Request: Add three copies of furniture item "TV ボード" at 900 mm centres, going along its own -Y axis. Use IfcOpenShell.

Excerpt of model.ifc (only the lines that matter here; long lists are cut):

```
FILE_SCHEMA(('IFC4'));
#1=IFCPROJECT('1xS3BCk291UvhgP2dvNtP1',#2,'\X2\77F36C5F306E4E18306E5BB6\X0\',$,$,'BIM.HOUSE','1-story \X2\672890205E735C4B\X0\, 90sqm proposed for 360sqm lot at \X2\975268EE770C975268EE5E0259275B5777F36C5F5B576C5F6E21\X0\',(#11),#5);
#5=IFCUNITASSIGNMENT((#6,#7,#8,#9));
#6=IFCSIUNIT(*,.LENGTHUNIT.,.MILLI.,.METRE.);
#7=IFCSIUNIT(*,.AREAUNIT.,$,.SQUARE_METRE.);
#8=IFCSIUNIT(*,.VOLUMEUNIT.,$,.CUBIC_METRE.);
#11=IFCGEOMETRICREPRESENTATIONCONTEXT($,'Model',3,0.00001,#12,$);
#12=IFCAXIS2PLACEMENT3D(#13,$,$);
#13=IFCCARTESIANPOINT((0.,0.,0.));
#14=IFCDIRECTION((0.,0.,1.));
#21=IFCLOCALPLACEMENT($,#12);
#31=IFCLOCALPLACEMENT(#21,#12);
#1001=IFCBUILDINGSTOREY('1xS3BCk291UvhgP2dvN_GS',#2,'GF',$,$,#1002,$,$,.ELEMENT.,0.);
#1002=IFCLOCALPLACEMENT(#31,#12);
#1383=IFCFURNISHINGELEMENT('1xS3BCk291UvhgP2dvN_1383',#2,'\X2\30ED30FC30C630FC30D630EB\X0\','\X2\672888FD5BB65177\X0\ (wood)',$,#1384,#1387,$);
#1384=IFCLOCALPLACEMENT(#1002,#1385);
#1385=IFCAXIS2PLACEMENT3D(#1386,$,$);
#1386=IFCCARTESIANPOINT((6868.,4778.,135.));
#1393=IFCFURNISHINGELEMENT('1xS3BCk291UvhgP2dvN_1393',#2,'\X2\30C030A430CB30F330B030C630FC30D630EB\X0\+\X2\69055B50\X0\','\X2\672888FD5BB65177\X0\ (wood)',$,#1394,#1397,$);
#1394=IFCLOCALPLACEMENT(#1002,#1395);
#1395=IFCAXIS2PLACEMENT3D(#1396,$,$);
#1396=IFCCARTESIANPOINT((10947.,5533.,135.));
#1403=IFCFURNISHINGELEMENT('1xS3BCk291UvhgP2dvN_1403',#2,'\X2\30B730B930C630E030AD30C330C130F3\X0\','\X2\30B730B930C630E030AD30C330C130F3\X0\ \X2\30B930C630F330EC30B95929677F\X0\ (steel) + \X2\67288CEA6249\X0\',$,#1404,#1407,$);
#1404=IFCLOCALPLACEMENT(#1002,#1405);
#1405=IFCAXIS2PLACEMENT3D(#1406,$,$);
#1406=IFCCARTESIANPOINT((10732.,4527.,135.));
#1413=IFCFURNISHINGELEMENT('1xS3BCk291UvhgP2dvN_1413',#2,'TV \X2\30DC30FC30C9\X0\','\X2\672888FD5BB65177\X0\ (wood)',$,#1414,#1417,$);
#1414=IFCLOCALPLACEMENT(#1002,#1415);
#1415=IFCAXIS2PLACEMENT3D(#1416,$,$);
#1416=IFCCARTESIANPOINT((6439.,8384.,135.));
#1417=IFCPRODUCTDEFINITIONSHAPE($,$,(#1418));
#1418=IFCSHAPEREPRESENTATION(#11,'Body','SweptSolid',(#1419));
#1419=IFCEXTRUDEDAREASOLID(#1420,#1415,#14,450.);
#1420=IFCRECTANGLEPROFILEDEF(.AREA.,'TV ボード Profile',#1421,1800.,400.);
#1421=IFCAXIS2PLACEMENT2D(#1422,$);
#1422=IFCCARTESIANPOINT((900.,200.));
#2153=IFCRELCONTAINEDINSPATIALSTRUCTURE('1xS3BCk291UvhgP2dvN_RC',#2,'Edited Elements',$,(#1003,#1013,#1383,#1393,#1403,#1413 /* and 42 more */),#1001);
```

```python
import ifcopenshell
import ifcopenshell.api.geometry
import ifcopenshell.api.root
import ifcopenshell.util.element
import ifcopenshell.util.placement
import ifcopenshell.util.unit

model = ifcopenshell.open("model.ifc")
unit_scale = ifcopenshell.util.unit.calculate_unit_scale(model)


def reuse_history(source, copy):
    """copy_class also copies each property set's owner history, people and application; keep the originals."""
    for rel in copy.IsDefinedBy:
        if rel.is_a("IfcRelDefinesByProperties") and (history := rel.RelatingPropertyDefinition.OwnerHistory):
            rel.RelatingPropertyDefinition.OwnerHistory = source.OwnerHistory
            ifcopenshell.util.element.remove_deep2(model, history)


source = model.by_guid("1xS3BCk291UvhgP2dvN_1413")
base = ifcopenshell.util.placement.get_local_placement(source.ObjectPlacement)
step = -base[:3, 1] * 0.9 / unit_scale

for i in range(1, 4):
    copy = ifcopenshell.api.root.copy_class(model, product=source)
    copy.Representation = ifcopenshell.util.element.copy_deep(
        model, source.Representation, exclude=["IfcGeometricRepresentationContext", "IfcRepresentationMap"]
    )
    reuse_history(source, copy)
    matrix = base.copy()
    matrix[:3, 3] += i * step
    print("added at", matrix[:3, 3].round(3) + 0.0)
    ifcopenshell.api.geometry.edit_object_placement(model, product=copy, matrix=matrix, is_si=False)

model.write("model_updated.ifc")
```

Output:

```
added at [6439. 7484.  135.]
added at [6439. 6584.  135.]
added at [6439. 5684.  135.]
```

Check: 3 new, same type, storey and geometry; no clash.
